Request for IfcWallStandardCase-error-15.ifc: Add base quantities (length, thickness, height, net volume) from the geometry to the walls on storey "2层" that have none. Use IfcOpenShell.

First a look at what the model holds.

```python
import ifcopenshell
import ifcopenshell.util.element
import ifcopenshell.util.unit

model = ifcopenshell.open("IfcWallStandardCase-error-15.ifc")
print(model.schema)
for unit_type in ("LENGTHUNIT", "AREAUNIT", "VOLUMEUNIT"):
    print(unit_type, ifcopenshell.util.unit.calculate_unit_scale(model, unit_type))
storey = next(s for s in model.by_type("IfcBuildingStorey") if s.Name == "2层")
walls = [e for e in ifcopenshell.util.element.get_decomposition(storey) if e.is_a("IfcWall")]
for e in sorted(walls, key=lambda e: e.id()):
    print(e.id(), e.is_a(), e.Name, list(ifcopenshell.util.element.get_psets(e, qtos_only=True)), sep=" | ")
```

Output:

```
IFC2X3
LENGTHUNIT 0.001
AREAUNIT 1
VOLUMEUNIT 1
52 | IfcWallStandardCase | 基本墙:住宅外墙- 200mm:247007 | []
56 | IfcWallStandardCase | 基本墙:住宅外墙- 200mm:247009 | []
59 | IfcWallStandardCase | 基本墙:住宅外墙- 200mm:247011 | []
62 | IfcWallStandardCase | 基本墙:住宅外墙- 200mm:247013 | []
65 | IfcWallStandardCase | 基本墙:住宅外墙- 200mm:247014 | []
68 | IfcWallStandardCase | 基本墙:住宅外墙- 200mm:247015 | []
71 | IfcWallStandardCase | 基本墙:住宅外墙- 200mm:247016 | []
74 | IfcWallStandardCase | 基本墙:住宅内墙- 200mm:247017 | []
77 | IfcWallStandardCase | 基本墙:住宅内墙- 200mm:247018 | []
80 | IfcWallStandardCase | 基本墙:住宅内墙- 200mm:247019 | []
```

```python
import ifcopenshell
import ifcopenshell.api.pset
import ifcopenshell.geom
import ifcopenshell.util.element
import ifcopenshell.util.shape
import ifcopenshell.util.unit

model = ifcopenshell.open("IfcWallStandardCase-error-15.ifc")
unit_scale = ifcopenshell.util.unit.calculate_unit_scale(model)
volume_scale = ifcopenshell.util.unit.calculate_unit_scale(model, "VOLUMEUNIT")
settings = ifcopenshell.geom.settings()

storey = next(s for s in model.by_type("IfcBuildingStorey") if s.Name == "2层")
walls = [e for e in ifcopenshell.util.element.get_decomposition(storey) if e.is_a("IfcWall")]

for e in sorted(walls, key=lambda e: e.id()):
    if ifcopenshell.util.element.get_psets(e, qtos_only=True, should_inherit=False):
        continue
    # Geometry comes back in metres, in the element's own axes.
    shape = ifcopenshell.geom.create_shape(settings, e)
    values = {
        "Length": ifcopenshell.util.shape.get_x(shape.geometry) / unit_scale,
        "Width": ifcopenshell.util.shape.get_y(shape.geometry) / unit_scale,
        "Height": ifcopenshell.util.shape.get_z(shape.geometry) / unit_scale,
        "NetVolume": ifcopenshell.util.shape.get_volume(shape.geometry) / volume_scale,
    }
    qto = ifcopenshell.api.pset.add_qto(model, product=e, name="BaseQuantities")
    ifcopenshell.api.pset.edit_qto(model, qto=qto, properties=values)
    print(e.id(), {k: round(v, 3) for k, v in values.items()})

model.write("IfcWallStandardCase-error-15-out.ifc")
```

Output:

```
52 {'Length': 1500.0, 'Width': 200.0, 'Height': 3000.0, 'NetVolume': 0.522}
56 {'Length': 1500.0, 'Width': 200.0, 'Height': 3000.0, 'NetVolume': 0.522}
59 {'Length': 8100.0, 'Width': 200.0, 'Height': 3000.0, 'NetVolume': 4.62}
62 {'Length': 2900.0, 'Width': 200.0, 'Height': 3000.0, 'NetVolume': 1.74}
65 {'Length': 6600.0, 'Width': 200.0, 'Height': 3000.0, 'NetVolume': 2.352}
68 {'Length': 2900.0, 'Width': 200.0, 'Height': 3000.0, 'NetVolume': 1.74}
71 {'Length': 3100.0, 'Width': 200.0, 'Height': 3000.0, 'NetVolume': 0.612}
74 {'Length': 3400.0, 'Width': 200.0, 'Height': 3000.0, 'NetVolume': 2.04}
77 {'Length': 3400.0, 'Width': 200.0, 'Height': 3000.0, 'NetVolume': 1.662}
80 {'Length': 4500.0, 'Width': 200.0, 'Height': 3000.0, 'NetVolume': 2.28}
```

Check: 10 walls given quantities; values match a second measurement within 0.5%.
